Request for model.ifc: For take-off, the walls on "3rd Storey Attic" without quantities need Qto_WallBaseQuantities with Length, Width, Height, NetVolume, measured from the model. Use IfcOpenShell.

First a look at what the model holds.

```python
import ifcopenshell
import ifcopenshell.util.element
import ifcopenshell.util.unit

model = ifcopenshell.open("model.ifc")
print(model.schema)
for unit_type in ("LENGTHUNIT", "AREAUNIT", "VOLUMEUNIT"):
    print(unit_type, ifcopenshell.util.unit.calculate_unit_scale(model, unit_type))
storey = next(s for s in model.by_type("IfcBuildingStorey") if s.Name == "3rd Storey Attic")
walls = [e for e in ifcopenshell.util.element.get_decomposition(storey) if e.is_a("IfcWall")]
for e in sorted(walls, key=lambda e: e.id()):
    print(e.id(), e.is_a(), e.Name, list(ifcopenshell.util.element.get_psets(e, qtos_only=True)), sep=" | ")
```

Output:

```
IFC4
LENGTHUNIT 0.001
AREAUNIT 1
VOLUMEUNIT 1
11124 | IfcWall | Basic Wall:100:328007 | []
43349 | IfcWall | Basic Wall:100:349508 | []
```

```python
import ifcopenshell
import ifcopenshell.api.pset
import ifcopenshell.geom
import ifcopenshell.util.element
import ifcopenshell.util.shape
import ifcopenshell.util.unit

model = ifcopenshell.open("model.ifc")
unit_scale = ifcopenshell.util.unit.calculate_unit_scale(model)
volume_scale = ifcopenshell.util.unit.calculate_unit_scale(model, "VOLUMEUNIT")
settings = ifcopenshell.geom.settings()

storey = next(s for s in model.by_type("IfcBuildingStorey") if s.Name == "3rd Storey Attic")
walls = [e for e in ifcopenshell.util.element.get_decomposition(storey) if e.is_a("IfcWall")]

for e in sorted(walls, key=lambda e: e.id()):
    if ifcopenshell.util.element.get_psets(e, qtos_only=True, should_inherit=False):
        continue
    # Geometry comes back in metres, in the element's own axes.
    shape = ifcopenshell.geom.create_shape(settings, e)
    values = {
        "Length": ifcopenshell.util.shape.get_x(shape.geometry) / unit_scale,
        "Width": ifcopenshell.util.shape.get_y(shape.geometry) / unit_scale,
        "Height": ifcopenshell.util.shape.get_z(shape.geometry) / unit_scale,
        "NetVolume": ifcopenshell.util.shape.get_volume(shape.geometry) / volume_scale,
    }
    qto = ifcopenshell.api.pset.add_qto(model, product=e, name="Qto_WallBaseQuantities")
    ifcopenshell.api.pset.edit_qto(model, qto=qto, properties=values)
    print(e.id(), {k: round(v, 3) for k, v in values.items()})

model.write("model-out.ifc")
```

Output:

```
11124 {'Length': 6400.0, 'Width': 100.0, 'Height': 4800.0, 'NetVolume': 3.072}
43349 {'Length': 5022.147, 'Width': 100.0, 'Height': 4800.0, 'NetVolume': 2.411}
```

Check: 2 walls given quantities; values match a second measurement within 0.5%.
